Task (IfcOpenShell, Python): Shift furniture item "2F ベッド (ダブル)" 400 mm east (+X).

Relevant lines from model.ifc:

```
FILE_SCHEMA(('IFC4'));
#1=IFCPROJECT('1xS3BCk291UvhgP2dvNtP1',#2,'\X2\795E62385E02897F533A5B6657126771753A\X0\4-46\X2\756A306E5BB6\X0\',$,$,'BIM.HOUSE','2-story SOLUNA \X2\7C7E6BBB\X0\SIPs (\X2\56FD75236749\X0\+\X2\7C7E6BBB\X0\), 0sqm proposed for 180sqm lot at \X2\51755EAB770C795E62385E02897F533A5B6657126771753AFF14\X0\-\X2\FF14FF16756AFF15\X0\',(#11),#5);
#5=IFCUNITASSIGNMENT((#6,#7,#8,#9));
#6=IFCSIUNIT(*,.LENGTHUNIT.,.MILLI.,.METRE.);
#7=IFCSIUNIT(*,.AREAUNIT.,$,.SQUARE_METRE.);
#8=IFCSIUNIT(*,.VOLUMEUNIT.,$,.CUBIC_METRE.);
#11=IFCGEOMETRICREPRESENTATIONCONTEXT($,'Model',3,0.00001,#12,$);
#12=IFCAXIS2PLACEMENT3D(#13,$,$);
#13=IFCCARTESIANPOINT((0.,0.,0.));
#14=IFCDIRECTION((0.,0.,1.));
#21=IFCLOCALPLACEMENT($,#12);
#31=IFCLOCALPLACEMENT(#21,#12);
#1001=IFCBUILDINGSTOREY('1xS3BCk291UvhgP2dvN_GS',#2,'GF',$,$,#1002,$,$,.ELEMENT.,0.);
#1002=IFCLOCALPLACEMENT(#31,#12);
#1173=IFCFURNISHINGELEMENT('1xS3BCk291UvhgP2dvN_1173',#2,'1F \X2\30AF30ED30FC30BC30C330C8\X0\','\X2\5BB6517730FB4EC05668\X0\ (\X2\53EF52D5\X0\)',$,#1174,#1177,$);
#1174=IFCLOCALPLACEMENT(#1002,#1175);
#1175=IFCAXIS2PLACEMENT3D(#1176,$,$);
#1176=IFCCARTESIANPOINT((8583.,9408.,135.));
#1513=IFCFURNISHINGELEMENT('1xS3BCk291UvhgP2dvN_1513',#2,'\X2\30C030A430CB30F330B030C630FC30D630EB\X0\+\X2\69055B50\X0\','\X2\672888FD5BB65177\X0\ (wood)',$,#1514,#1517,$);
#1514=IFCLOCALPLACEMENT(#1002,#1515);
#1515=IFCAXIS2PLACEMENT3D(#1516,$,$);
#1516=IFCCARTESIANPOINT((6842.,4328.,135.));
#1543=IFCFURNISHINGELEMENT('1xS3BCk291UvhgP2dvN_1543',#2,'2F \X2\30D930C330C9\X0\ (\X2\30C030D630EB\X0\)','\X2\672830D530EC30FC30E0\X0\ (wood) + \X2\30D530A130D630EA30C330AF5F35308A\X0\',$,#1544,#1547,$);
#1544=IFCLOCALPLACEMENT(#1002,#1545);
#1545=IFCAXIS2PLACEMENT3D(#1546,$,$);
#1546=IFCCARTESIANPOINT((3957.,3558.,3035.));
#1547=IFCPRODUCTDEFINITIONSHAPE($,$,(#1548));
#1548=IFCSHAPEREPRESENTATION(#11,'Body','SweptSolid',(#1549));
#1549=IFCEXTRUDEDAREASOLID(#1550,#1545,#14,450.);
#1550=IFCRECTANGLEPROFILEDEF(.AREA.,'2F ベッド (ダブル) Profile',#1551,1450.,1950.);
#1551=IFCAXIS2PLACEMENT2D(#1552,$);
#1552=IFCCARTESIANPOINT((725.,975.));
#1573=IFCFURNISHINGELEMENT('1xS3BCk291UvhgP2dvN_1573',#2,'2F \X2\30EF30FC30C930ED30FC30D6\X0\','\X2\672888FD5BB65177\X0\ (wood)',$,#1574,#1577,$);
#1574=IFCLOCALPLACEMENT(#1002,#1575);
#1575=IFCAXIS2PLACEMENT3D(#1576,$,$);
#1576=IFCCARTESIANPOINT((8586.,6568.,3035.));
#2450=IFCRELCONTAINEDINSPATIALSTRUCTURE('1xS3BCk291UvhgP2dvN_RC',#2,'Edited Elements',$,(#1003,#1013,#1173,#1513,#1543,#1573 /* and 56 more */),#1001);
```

```python
import ifcopenshell
import ifcopenshell.api.geometry
import ifcopenshell.util.placement
import ifcopenshell.util.unit

model = ifcopenshell.open("model.ifc")
unit_scale = ifcopenshell.util.unit.calculate_unit_scale(model)

item = model.by_guid("1xS3BCk291UvhgP2dvN_1543")
matrix = ifcopenshell.util.placement.get_local_placement(item.ObjectPlacement)
matrix[0, 3] += 0.4 / unit_scale
ifcopenshell.api.geometry.edit_object_placement(model, product=item, matrix=matrix, is_si=False)

print(ifcopenshell.util.placement.get_local_placement(item.ObjectPlacement).round(3) + 0.0)

model.write("model-out.ifc")
```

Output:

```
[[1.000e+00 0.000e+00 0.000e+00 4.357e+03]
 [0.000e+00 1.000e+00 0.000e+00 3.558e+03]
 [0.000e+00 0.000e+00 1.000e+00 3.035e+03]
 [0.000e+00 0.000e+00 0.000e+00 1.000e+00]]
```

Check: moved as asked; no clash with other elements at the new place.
